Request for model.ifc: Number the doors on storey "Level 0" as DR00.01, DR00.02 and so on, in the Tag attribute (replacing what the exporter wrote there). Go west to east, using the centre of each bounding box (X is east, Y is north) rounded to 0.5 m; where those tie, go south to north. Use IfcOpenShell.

First a look at what the model holds.

```python
import ifcopenshell
import ifcopenshell.util.element
import ifcopenshell.util.placement

model = ifcopenshell.open("model.ifc")
print(model.schema)
storey = next(s for s in model.by_type("IfcBuildingStorey") if s.Name == "Level 0")
doors = [e for e in ifcopenshell.util.element.get_decomposition(storey) if e.is_a("IfcDoor")]
for e in sorted(doors, key=lambda e: e.id()):
    origin = ifcopenshell.util.placement.get_local_placement(e.ObjectPlacement)[:3, 3]
    print(e.id(), e.Tag, e.Name, origin.round(2) + 0.0, sep=" | ")
```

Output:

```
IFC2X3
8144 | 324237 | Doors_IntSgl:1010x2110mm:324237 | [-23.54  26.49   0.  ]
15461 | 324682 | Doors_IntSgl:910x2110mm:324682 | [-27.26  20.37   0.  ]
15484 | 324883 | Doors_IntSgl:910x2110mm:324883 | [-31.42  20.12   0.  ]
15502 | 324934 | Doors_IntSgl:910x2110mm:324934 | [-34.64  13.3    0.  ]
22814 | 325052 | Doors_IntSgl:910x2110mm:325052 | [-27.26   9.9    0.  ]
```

```python
import ifcopenshell
import ifcopenshell.geom
import ifcopenshell.util.element
import ifcopenshell.util.shape

model = ifcopenshell.open("model.ifc")
settings = ifcopenshell.geom.settings()
settings.set("use-world-coords", True)


def centre(element):
    shape = ifcopenshell.geom.create_shape(settings, element)
    return ifcopenshell.util.shape.get_bbox_centroid(shape.geometry)


storey = next(s for s in model.by_type("IfcBuildingStorey") if s.Name == "Level 0")
doors = [e for e in ifcopenshell.util.element.get_decomposition(storey) if e.is_a("IfcDoor")]

# Insertion points can sit at a corner or the storey origin, so sort by the geometry (in metres).
centres = {e: centre(e) for e in doors}
doors.sort(key=lambda e: (round(centres[e][0] / 0.5), centres[e][1]))

for i, e in enumerate(doors, start=1):
    number = f"DR00.{i:02d}"
    e.Tag = number
    print(e.id(), number)

model.write("model_edited.ifc")
```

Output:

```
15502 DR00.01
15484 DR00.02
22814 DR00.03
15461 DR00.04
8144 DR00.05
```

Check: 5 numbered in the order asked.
